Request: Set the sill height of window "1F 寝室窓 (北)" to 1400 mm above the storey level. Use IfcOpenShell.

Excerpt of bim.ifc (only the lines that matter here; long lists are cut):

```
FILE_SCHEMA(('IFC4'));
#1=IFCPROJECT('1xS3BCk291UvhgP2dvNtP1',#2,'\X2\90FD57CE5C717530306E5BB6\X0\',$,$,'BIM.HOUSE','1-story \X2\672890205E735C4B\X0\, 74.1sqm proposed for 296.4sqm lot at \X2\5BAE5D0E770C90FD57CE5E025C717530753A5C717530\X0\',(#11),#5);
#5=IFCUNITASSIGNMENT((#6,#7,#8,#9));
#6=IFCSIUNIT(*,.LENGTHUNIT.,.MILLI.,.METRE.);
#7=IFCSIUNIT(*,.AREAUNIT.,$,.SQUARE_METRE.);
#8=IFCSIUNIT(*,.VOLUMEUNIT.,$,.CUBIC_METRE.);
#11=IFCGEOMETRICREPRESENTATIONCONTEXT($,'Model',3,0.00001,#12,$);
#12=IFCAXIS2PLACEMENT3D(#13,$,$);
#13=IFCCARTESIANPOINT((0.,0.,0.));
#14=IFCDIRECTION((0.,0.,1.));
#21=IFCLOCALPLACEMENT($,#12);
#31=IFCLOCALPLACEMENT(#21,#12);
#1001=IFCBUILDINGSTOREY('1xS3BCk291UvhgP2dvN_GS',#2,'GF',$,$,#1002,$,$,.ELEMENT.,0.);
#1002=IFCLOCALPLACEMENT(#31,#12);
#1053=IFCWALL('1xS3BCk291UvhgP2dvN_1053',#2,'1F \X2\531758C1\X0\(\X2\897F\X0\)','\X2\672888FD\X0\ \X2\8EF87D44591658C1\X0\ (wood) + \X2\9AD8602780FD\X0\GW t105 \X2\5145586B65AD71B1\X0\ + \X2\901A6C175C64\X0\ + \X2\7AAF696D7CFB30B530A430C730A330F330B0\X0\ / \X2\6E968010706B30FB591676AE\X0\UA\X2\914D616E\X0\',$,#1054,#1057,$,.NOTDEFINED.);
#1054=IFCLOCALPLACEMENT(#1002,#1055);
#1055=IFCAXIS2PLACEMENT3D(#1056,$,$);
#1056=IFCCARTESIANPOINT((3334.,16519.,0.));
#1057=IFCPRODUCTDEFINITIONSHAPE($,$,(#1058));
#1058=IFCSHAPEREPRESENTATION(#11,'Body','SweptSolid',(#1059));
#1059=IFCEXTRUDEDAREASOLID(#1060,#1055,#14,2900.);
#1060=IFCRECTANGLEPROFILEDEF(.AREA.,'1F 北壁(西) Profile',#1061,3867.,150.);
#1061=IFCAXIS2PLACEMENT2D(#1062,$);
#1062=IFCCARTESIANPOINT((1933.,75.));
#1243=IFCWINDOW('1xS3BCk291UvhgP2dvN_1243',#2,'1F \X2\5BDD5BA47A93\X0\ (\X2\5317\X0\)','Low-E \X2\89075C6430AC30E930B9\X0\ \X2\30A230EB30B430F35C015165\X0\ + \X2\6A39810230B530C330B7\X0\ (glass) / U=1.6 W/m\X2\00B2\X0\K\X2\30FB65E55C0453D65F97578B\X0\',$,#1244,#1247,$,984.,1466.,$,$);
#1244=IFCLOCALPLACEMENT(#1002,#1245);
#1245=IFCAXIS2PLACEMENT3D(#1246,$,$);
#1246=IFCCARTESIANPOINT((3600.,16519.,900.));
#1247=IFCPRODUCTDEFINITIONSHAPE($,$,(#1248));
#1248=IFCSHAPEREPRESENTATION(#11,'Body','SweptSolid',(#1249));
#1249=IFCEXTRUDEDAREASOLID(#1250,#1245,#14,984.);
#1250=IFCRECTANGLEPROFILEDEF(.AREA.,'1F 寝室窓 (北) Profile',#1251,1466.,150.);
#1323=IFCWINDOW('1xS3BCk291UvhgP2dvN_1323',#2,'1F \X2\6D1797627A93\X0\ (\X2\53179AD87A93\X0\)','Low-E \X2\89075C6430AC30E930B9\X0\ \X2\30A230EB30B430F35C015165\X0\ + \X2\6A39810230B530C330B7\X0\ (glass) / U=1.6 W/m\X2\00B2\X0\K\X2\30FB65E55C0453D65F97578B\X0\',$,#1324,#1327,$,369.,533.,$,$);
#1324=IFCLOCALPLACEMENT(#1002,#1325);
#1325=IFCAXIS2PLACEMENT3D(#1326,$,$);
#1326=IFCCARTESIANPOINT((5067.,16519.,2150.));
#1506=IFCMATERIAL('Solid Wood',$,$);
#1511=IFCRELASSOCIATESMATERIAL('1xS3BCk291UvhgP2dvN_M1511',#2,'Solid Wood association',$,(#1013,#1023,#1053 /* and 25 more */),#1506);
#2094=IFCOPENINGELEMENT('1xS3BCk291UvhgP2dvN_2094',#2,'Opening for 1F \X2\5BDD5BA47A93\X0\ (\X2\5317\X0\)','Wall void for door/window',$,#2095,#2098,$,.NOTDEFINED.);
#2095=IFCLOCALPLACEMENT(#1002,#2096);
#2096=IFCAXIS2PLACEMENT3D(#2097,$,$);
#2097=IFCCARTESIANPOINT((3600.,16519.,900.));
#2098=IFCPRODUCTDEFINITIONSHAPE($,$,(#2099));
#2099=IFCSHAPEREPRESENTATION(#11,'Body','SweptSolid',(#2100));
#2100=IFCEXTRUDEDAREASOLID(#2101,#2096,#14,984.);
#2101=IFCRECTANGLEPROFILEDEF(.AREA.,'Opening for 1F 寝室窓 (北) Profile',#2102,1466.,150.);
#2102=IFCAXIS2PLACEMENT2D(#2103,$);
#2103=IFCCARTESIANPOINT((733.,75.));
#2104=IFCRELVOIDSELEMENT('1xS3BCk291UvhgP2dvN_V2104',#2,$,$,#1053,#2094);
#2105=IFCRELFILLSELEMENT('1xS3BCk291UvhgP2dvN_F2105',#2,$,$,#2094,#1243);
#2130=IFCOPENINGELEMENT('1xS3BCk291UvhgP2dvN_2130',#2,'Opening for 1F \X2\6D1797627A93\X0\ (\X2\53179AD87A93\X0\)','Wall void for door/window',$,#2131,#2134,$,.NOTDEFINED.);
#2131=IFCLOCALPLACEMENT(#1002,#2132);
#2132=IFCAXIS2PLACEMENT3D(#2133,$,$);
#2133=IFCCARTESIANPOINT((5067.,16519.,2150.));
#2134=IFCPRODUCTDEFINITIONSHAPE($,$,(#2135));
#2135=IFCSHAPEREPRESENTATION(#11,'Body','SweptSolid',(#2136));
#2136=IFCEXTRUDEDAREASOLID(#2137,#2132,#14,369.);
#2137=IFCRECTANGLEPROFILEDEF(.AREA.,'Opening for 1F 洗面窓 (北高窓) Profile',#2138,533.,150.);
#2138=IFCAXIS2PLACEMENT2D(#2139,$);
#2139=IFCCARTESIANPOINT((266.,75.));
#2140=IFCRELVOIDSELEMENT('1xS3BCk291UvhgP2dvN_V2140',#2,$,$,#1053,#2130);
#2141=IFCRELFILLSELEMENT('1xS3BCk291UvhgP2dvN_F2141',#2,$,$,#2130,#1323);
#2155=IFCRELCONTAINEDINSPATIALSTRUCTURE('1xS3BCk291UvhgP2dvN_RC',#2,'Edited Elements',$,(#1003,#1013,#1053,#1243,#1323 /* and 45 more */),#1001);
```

```python
import numpy as np
import ifcopenshell
import ifcopenshell.api.geometry
import ifcopenshell.geom
import ifcopenshell.util.element
import ifcopenshell.util.placement
import ifcopenshell.util.shape
import ifcopenshell.util.unit

model = ifcopenshell.open("bim.ifc")
unit_scale = ifcopenshell.util.unit.calculate_unit_scale(model)

window = model.by_guid("1xS3BCk291UvhgP2dvN_1243")
opening = window.FillsVoids[0].RelatingOpeningElement
storey = ifcopenshell.util.element.get_container(window, ifc_class="IfcBuildingStorey")
level = ifcopenshell.util.placement.get_local_placement(storey.ObjectPlacement)[2, 3]

# The opening's origin need not be at the sill, so measure its lowest point.
shape = ifcopenshell.geom.create_shape(ifcopenshell.geom.settings(), opening)
bottom = ifcopenshell.util.shape.get_shape_bottom_elevation(shape, shape.geometry) / unit_scale
dz = level + 1400.0 - bottom

shift = np.array([0.0, 0.0, dz])
# The window is not placed relative to its opening, so move both.
for product in (opening, window):
    matrix = ifcopenshell.util.placement.get_local_placement(product.ObjectPlacement)
    matrix[:3, 3] += shift
    ifcopenshell.api.geometry.edit_object_placement(model, product=product, matrix=matrix, is_si=False)

print(f"moved by {dz * unit_scale:+.3f} m")

model.write("bim_edited.ifc")
```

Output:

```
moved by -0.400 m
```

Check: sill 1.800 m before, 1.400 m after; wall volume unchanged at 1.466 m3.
